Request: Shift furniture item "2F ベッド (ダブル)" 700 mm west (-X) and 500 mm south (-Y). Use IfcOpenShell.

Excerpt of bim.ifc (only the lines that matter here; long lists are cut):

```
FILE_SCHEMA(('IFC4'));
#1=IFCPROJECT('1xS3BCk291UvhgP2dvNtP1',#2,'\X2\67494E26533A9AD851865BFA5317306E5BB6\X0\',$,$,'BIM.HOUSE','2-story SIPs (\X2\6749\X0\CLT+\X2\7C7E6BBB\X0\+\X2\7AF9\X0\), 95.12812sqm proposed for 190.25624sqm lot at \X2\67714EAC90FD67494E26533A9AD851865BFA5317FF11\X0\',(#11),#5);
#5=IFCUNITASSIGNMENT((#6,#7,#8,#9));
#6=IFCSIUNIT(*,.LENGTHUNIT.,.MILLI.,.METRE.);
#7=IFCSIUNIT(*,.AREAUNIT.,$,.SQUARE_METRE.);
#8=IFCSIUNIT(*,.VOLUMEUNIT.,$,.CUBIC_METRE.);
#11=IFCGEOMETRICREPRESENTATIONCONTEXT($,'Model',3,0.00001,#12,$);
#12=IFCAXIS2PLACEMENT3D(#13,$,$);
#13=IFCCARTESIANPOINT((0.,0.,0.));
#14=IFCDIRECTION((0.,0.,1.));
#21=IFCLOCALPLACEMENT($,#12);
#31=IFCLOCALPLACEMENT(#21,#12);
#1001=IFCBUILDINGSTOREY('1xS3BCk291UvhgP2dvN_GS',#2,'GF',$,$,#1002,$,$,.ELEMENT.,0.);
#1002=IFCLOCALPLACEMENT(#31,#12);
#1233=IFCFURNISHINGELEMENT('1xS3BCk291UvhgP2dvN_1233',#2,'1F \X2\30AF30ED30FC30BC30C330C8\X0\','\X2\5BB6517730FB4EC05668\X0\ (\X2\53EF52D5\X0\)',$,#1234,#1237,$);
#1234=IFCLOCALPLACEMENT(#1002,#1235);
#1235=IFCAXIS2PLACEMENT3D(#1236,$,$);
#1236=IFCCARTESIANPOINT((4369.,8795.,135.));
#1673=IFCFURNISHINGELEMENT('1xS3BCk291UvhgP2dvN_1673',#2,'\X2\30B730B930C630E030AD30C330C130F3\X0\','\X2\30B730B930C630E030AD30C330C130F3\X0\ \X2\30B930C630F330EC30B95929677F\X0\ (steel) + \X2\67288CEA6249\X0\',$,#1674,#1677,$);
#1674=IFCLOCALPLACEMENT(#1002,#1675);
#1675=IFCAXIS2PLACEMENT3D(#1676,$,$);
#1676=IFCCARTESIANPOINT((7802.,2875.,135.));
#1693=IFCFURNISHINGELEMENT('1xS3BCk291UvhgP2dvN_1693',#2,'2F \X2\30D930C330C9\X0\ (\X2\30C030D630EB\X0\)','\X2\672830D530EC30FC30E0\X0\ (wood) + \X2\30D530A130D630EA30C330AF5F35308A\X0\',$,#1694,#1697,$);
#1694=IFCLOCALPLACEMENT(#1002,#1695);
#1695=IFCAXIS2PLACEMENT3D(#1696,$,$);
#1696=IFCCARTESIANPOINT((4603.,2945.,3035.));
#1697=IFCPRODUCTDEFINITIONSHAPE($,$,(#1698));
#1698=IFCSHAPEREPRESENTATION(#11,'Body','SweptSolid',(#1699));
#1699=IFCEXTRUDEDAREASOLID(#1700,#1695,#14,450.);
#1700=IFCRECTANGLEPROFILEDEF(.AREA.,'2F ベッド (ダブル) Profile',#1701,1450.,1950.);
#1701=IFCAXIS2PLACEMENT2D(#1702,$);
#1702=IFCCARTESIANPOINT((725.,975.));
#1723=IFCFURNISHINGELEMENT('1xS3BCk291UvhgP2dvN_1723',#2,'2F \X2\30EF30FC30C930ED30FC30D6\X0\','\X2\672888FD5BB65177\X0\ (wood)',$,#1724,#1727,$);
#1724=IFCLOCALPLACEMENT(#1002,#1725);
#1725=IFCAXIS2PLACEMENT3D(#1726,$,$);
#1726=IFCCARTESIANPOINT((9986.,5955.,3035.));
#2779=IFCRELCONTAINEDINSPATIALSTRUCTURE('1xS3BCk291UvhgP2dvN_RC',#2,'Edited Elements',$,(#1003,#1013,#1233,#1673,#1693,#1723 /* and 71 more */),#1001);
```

```python
import ifcopenshell
import ifcopenshell.api.geometry
import ifcopenshell.util.placement

model = ifcopenshell.open("bim.ifc")

item = model.by_guid("1xS3BCk291UvhgP2dvN_1693")
matrix = ifcopenshell.util.placement.get_local_placement(item.ObjectPlacement)
matrix[0, 3] -= 700.0
matrix[1, 3] -= 500.0
ifcopenshell.api.geometry.edit_object_placement(model, product=item, matrix=matrix, is_si=False)

print(ifcopenshell.util.placement.get_local_placement(item.ObjectPlacement).round(3) + 0.0)

model.write("bim_edited.ifc")
```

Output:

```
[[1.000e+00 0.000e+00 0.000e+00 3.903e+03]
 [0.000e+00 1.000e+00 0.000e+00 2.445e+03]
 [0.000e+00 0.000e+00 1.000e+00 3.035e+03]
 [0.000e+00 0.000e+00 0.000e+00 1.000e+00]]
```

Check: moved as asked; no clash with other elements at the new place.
